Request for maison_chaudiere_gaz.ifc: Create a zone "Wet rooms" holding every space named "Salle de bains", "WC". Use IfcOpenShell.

First a look at what the model holds.

```python
import ifcopenshell

model = ifcopenshell.open("maison_chaudiere_gaz.ifc")
print(model.schema)
seen = {}
for space in model.by_type("IfcSpace"):
    seen[space.LongName] = seen.get(space.LongName, 0) + 1
for name, count in sorted(seen.items(), key=str):
    print(count, "x", name)
print("zones:", [z.Name for z in model.by_type("IfcZone")][:20])
```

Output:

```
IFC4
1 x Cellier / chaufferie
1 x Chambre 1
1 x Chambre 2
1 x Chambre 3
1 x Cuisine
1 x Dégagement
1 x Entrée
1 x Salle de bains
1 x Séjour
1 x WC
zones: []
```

```python
import ifcopenshell
import ifcopenshell.api.group
import ifcopenshell.api.root

model = ifcopenshell.open("maison_chaudiere_gaz.ifc")

names = {"Salle de bains", "WC"}
spaces = [s for s in model.by_type("IfcSpace") if s.LongName in names]

zone = ifcopenshell.api.root.create_entity(model, ifc_class="IfcZone", name="Wet rooms")
ifcopenshell.api.group.assign_group(model, products=spaces, group=zone)
print(len(spaces), "spaces in", zone.Name)

model.write("maison_chaudiere_gaz_updated.ifc")
```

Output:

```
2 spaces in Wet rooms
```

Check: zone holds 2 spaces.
